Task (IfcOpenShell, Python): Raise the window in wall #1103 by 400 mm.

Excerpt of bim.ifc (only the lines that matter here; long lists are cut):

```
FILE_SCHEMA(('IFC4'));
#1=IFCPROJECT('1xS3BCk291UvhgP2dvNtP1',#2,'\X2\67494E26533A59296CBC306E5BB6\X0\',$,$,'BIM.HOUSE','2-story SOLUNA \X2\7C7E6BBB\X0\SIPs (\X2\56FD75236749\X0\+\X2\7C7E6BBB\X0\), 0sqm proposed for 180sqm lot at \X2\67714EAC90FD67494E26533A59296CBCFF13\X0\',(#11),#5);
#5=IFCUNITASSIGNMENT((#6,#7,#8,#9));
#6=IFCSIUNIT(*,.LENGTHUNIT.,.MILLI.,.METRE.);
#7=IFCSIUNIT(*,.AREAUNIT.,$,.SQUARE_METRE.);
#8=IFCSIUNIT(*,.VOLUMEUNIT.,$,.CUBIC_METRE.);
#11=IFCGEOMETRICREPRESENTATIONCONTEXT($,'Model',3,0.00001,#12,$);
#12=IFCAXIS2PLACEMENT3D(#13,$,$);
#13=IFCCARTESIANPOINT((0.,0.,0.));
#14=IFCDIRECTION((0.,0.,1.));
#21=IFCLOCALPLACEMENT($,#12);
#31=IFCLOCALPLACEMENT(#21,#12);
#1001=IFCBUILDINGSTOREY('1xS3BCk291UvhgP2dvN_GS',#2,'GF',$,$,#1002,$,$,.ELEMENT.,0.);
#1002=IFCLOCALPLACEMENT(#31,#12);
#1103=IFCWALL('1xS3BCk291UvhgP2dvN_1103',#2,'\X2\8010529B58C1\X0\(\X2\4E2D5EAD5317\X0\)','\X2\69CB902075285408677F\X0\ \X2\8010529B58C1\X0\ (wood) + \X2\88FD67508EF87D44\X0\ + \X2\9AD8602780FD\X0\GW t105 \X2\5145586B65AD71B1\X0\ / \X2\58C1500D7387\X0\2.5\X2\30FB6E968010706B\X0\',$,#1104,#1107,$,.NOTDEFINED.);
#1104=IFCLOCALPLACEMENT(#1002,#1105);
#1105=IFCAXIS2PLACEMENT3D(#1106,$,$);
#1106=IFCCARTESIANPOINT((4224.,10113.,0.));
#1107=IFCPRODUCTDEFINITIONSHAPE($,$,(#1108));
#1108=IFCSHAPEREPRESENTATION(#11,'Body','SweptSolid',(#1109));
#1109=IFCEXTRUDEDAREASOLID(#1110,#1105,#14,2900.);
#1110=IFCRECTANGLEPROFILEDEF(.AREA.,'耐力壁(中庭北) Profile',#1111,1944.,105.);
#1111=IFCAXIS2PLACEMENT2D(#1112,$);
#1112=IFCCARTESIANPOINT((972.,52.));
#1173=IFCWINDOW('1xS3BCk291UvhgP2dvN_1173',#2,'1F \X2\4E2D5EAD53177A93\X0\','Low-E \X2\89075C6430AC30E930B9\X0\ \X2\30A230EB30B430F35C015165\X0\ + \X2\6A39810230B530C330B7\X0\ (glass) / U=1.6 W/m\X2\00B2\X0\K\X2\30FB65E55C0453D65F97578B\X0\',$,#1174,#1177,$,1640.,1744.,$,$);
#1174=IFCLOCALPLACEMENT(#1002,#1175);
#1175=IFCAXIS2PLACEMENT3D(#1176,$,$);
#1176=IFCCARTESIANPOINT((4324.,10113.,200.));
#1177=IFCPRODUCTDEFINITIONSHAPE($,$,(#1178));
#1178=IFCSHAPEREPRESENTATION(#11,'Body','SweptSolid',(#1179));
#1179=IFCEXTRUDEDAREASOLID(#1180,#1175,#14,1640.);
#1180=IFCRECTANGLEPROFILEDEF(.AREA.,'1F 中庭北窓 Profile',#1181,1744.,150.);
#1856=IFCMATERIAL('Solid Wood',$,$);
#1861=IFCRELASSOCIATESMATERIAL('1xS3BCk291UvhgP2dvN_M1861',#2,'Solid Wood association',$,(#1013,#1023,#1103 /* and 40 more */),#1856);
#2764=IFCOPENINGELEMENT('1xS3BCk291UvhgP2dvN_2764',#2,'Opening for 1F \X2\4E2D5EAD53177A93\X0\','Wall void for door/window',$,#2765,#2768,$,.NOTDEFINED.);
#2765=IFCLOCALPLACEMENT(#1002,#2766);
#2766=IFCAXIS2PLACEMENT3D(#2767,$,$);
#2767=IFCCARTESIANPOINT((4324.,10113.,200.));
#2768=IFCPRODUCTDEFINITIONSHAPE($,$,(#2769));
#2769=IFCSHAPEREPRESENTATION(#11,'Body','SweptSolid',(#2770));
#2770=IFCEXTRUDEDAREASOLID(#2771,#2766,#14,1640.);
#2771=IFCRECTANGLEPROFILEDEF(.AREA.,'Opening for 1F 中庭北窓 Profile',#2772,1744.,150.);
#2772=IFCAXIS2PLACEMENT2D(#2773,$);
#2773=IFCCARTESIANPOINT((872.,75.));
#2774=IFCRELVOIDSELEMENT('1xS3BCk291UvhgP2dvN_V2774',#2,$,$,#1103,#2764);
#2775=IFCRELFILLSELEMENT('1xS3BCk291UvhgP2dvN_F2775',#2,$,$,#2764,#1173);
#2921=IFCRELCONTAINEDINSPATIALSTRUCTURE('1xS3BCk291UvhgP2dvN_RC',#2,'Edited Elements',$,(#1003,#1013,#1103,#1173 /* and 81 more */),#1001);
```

```python
import numpy as np
import ifcopenshell
import ifcopenshell.api.geometry
import ifcopenshell.util.placement
import ifcopenshell.util.unit

model = ifcopenshell.open("bim.ifc")
unit_scale = ifcopenshell.util.unit.calculate_unit_scale(model)

window = model.by_guid("1xS3BCk291UvhgP2dvN_1173")
opening = window.FillsVoids[0].RelatingOpeningElement
dz = 0.4 / unit_scale

shift = np.array([0.0, 0.0, dz])
# The window is not placed relative to its opening, so move both.
for product in (opening, window):
    matrix = ifcopenshell.util.placement.get_local_placement(product.ObjectPlacement)
    matrix[:3, 3] += shift
    ifcopenshell.api.geometry.edit_object_placement(model, product=product, matrix=matrix, is_si=False)

print(f"moved by {dz * unit_scale:+.3f} m")

model.write("bim_updated.ifc")
```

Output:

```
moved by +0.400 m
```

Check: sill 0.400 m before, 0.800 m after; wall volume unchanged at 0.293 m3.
